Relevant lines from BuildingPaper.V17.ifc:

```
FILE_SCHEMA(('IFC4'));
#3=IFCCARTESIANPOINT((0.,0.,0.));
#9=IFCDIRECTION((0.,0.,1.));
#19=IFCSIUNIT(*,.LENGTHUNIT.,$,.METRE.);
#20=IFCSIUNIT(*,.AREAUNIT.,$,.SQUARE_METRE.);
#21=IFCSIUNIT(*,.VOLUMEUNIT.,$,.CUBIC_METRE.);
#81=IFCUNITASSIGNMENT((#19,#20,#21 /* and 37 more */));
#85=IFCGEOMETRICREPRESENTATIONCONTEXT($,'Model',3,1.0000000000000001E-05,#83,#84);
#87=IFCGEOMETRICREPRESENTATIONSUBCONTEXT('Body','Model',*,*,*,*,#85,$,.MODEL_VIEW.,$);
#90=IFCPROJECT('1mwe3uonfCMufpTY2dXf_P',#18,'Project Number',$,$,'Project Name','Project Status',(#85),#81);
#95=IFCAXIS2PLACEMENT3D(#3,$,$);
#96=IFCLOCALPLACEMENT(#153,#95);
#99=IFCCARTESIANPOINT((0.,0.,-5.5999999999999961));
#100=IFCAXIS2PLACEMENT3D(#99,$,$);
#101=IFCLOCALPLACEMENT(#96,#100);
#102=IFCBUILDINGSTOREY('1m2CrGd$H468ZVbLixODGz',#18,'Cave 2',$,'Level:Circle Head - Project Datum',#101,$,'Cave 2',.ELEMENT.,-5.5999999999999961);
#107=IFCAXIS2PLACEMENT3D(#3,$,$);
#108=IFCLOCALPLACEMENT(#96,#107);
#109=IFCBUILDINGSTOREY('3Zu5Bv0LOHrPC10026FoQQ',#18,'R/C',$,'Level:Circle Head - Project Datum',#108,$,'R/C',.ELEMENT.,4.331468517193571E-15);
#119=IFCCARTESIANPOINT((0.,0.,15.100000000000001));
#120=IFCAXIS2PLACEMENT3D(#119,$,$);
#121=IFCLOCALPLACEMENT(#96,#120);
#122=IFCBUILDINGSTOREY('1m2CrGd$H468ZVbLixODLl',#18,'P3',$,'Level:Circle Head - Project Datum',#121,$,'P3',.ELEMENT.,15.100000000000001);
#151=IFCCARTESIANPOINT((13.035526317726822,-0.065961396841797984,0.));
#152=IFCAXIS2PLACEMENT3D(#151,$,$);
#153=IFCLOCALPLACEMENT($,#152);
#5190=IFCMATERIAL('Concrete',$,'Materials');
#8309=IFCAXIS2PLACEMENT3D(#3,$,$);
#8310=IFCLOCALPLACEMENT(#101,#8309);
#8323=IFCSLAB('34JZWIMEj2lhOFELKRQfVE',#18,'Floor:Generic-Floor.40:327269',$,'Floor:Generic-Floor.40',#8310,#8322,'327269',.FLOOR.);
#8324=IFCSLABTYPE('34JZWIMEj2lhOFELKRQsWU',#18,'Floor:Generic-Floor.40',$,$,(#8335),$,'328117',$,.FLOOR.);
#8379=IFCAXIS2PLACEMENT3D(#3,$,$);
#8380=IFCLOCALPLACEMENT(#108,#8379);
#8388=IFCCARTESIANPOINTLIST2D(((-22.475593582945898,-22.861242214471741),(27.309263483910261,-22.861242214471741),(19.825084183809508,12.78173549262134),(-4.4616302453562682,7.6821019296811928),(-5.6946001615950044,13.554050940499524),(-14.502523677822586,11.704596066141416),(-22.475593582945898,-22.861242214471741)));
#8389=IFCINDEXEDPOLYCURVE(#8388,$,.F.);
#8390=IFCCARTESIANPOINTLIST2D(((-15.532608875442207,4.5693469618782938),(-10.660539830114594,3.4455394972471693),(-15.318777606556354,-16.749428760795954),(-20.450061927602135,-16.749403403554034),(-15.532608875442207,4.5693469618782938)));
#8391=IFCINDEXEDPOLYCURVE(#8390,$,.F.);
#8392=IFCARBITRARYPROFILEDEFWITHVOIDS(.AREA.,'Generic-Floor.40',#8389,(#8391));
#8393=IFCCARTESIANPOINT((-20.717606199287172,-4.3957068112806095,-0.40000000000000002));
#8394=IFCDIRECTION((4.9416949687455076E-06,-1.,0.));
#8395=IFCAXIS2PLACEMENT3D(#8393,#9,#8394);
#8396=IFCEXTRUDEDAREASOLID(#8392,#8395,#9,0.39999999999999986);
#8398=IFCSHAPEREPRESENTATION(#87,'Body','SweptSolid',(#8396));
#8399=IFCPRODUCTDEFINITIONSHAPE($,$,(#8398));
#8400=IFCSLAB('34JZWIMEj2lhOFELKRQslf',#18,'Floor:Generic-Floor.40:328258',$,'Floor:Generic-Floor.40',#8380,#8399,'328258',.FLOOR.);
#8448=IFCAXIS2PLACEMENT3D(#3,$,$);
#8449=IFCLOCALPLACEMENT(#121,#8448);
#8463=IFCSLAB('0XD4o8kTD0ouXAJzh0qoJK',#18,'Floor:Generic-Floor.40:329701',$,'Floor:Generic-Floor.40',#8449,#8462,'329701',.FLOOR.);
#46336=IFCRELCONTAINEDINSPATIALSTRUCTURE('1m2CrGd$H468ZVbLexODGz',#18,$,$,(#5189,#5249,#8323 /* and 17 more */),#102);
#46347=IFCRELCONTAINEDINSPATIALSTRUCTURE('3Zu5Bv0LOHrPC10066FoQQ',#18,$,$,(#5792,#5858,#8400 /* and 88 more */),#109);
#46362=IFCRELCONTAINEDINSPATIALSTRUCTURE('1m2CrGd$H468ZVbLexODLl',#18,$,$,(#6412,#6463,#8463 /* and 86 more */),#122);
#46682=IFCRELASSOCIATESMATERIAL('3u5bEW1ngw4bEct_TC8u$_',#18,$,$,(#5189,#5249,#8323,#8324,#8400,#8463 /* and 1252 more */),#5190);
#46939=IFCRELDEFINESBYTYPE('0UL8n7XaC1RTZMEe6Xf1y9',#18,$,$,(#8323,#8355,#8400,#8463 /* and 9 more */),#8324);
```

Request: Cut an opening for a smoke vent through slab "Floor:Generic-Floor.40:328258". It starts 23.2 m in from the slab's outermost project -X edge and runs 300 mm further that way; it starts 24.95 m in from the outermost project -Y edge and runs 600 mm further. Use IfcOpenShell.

```python
import numpy as np
import ifcopenshell
import ifcopenshell.api.feature
import ifcopenshell.api.geometry
import ifcopenshell.api.root
import ifcopenshell.geom
import ifcopenshell.util.placement
import ifcopenshell.util.representation
import ifcopenshell.util.shape
import ifcopenshell.util.unit

model = ifcopenshell.open("BuildingPaper.V17.ifc")
unit_scale = ifcopenshell.util.unit.calculate_unit_scale(model)
settings = ifcopenshell.geom.settings()


def volume(element):
    """Net volume in cubic metres, openings subtracted."""
    shape = ifcopenshell.geom.create_shape(settings, element)
    return ifcopenshell.util.shape.get_volume(shape.geometry)


slab = model.by_guid("34JZWIMEj2lhOFELKRQslf")
before = volume(slab)

# Extent in the slab's own axes, in metres. The edges named are its -X and -Y sides.
slab_shape = ifcopenshell.geom.create_shape(settings, slab)
vertices = ifcopenshell.util.shape.get_vertices(slab_shape.geometry)
x_min, y_min, bottom = vertices.min(axis=0)
top = vertices[:, 2].max()

opening = ifcopenshell.api.root.create_entity(model, ifc_class="IfcOpeningElement", name="Smoke vent opening", predefined_type="OPENING")
context = ifcopenshell.util.representation.get_context(model, "Model", "Body", "MODEL_VIEW")
width, depth = 0.3, 0.6
outline = [(0.0, 0.0), (width, 0.0), (width, depth), (0.0, depth), (0.0, 0.0)]
# Overshoot both faces by 50 mm so the cut is clean.
shape = ifcopenshell.api.geometry.add_slab_representation(
    model, context=context, depth=top - bottom + 0.1, polyline=outline
)
ifcopenshell.api.geometry.assign_representation(model, product=opening, representation=shape)

matrix = ifcopenshell.util.placement.get_local_placement(slab.ObjectPlacement)
matrix[:, 3] = matrix @ np.append(np.array([x_min + 23.2, y_min + 24.95, bottom - 0.05]) / unit_scale, 1.0)
ifcopenshell.api.geometry.edit_object_placement(model, product=opening, matrix=matrix, is_si=False)
ifcopenshell.api.feature.add_feature(model, feature=opening, element=slab)

after = volume(slab)

print(f"slab volume {before:.3f} -> {after:.3f} m3")

model.write("BuildingPaper.V17_edited.ifc")
```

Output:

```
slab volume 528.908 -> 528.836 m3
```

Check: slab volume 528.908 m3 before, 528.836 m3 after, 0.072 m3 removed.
